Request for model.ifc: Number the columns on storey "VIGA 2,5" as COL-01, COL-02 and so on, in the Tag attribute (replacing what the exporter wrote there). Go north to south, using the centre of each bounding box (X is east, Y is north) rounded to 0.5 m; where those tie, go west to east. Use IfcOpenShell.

First a look at what the model holds.

```python
import ifcopenshell
import ifcopenshell.util.element
import ifcopenshell.util.placement

model = ifcopenshell.open("model.ifc")
print(model.schema)
storey = next(s for s in model.by_type("IfcBuildingStorey") if s.Name == "VIGA 2,5")
columns = [e for e in ifcopenshell.util.element.get_decomposition(storey) if e.is_a("IfcColumn")]
for e in sorted(columns, key=lambda e: e.id()):
    origin = ifcopenshell.util.placement.get_local_placement(e.ObjectPlacement)[:3, 3]
    print(e.id(), e.Tag, e.Name, origin.round(2) + 0.0, sep=" | ")
```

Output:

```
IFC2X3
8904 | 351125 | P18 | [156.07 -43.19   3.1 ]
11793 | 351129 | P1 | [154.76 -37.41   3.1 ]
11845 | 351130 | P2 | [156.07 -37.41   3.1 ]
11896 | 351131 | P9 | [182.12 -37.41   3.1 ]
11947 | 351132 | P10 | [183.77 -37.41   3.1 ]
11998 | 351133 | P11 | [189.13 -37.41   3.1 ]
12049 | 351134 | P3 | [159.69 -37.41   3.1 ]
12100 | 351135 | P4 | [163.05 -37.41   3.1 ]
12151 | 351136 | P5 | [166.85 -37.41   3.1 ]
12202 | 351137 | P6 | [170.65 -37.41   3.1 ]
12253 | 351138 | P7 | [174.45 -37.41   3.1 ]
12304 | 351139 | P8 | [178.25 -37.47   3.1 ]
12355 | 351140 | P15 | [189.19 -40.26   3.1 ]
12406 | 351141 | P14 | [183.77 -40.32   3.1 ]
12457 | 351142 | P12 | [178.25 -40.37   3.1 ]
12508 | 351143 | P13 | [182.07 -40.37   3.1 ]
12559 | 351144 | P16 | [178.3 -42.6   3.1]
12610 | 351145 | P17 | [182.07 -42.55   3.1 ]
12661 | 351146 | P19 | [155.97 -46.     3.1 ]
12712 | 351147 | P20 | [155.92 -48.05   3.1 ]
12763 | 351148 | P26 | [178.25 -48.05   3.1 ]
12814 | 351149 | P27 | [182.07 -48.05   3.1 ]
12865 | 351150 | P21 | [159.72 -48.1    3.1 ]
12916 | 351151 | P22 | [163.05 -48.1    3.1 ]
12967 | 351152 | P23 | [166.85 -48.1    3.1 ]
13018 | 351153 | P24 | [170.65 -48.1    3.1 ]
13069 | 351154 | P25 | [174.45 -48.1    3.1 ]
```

```python
import ifcopenshell
import ifcopenshell.geom
import ifcopenshell.util.element
import ifcopenshell.util.shape

model = ifcopenshell.open("model.ifc")
settings = ifcopenshell.geom.settings()
settings.set("use-world-coords", True)


def centre(element):
    shape = ifcopenshell.geom.create_shape(settings, element)
    return ifcopenshell.util.shape.get_bbox_centroid(shape.geometry)


storey = next(s for s in model.by_type("IfcBuildingStorey") if s.Name == "VIGA 2,5")
columns = [e for e in ifcopenshell.util.element.get_decomposition(storey) if e.is_a("IfcColumn")]

# Insertion points can sit at a corner or the storey origin, so sort by the geometry (in metres).
centres = {e: centre(e) for e in columns}
columns.sort(key=lambda e: (-round(centres[e][1] / 0.5), centres[e][0]))

for i, e in enumerate(columns, start=1):
    number = f"COL-{i:02d}"
    e.Tag = number
    print(e.id(), number)

model.write("model_updated.ifc")
```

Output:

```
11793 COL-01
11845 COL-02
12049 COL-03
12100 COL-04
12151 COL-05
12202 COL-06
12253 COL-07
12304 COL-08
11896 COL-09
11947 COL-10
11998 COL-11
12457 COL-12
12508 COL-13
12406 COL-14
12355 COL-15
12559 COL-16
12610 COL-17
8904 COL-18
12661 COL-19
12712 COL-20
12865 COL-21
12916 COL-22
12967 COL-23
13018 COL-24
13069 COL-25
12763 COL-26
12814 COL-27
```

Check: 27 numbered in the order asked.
